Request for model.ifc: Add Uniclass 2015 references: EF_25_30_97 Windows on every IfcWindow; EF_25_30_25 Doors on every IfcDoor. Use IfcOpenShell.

First a look at what the model holds.

```python
import ifcopenshell

model = ifcopenshell.open("model.ifc")
print(model.schema)
print("classifications:", [c.Name for c in model.by_type("IfcClassification")])
for ifc_class in ("IfcDoor", "IfcRoof", "IfcStair", "IfcWall", "IfcWindow"):
    print(ifc_class, len(model.by_type(ifc_class)))
```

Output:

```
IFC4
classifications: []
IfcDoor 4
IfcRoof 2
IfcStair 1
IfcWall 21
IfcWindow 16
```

```python
import ifcopenshell
import ifcopenshell.api.classification

model = ifcopenshell.open("model.ifc")

system = ifcopenshell.api.classification.add_classification(model, classification="Uniclass 2015")

codes = {
    "IfcWindow": ("EF_25_30_97", "Windows"),
    "IfcDoor": ("EF_25_30_25", "Doors"),
}
for ifc_class, (code, name) in codes.items():
    products = model.by_type(ifc_class)
    ifcopenshell.api.classification.add_reference(
        model, products=products, classification=system, identification=code, name=name
    )
    print(code, len(products))

model.write("model-out.ifc")
```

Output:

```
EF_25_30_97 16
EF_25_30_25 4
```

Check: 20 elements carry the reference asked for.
